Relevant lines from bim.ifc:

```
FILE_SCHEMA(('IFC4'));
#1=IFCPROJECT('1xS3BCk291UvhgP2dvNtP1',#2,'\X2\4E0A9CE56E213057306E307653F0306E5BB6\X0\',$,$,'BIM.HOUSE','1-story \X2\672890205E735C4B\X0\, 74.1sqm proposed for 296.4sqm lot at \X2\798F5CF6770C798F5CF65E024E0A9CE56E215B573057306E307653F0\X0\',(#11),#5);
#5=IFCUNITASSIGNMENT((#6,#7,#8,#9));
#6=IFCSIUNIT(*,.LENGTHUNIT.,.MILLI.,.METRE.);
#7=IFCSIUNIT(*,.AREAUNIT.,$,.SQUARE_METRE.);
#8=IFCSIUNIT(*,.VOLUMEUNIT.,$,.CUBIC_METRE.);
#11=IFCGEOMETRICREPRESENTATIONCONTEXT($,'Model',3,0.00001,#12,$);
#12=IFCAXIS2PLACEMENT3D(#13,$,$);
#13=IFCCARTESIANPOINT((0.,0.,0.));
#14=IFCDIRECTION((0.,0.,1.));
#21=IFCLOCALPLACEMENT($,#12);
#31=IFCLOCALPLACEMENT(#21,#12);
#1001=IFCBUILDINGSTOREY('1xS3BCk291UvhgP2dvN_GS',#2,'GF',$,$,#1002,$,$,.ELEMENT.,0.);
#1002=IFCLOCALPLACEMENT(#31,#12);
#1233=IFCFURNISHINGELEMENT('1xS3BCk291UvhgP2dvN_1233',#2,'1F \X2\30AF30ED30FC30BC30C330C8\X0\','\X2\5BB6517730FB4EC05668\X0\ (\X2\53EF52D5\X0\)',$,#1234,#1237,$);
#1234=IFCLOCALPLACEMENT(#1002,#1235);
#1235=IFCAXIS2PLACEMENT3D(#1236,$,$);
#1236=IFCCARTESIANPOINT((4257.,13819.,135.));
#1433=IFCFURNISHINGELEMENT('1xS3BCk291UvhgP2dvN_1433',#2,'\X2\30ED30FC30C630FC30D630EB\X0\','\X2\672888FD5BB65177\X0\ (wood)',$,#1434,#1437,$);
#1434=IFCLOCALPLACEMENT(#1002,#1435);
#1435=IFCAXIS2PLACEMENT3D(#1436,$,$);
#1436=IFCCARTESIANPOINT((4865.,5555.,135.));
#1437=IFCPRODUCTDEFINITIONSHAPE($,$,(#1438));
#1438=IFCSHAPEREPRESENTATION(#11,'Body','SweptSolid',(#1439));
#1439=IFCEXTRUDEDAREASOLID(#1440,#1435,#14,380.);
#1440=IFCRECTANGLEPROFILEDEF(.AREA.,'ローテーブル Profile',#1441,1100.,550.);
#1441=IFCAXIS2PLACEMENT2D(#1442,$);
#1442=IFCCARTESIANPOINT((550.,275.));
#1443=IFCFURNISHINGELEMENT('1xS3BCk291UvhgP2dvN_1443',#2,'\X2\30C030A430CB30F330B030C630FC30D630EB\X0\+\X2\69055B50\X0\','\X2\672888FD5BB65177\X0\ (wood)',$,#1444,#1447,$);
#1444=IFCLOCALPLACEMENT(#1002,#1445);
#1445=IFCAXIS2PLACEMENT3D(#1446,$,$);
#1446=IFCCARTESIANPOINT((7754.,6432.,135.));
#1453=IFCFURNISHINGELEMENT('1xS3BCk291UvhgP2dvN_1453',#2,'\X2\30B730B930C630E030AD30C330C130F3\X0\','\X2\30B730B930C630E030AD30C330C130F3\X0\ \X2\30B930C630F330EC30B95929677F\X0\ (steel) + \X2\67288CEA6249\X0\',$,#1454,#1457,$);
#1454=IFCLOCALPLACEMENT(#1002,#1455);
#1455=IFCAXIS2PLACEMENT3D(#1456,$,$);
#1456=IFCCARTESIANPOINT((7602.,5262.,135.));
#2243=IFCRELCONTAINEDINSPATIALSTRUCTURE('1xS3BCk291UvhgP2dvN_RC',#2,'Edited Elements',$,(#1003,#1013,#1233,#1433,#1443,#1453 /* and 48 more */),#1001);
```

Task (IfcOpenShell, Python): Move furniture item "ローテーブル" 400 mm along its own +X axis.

```python
import ifcopenshell
import ifcopenshell.api.geometry
import ifcopenshell.util.placement
import ifcopenshell.util.unit

model = ifcopenshell.open("bim.ifc")
unit_scale = ifcopenshell.util.unit.calculate_unit_scale(model)

item = model.by_guid("1xS3BCk291UvhgP2dvN_1433")
matrix = ifcopenshell.util.placement.get_local_placement(item.ObjectPlacement)
matrix[:3, 3] += matrix[:3, 0] * 0.4 / unit_scale
ifcopenshell.api.geometry.edit_object_placement(model, product=item, matrix=matrix, is_si=False)

print(ifcopenshell.util.placement.get_local_placement(item.ObjectPlacement).round(3) + 0.0)

model.write("bim_updated.ifc")
```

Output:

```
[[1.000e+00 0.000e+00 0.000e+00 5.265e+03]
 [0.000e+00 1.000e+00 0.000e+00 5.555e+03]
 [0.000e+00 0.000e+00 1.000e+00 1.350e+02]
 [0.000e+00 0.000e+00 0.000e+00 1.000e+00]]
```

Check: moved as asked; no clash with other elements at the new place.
